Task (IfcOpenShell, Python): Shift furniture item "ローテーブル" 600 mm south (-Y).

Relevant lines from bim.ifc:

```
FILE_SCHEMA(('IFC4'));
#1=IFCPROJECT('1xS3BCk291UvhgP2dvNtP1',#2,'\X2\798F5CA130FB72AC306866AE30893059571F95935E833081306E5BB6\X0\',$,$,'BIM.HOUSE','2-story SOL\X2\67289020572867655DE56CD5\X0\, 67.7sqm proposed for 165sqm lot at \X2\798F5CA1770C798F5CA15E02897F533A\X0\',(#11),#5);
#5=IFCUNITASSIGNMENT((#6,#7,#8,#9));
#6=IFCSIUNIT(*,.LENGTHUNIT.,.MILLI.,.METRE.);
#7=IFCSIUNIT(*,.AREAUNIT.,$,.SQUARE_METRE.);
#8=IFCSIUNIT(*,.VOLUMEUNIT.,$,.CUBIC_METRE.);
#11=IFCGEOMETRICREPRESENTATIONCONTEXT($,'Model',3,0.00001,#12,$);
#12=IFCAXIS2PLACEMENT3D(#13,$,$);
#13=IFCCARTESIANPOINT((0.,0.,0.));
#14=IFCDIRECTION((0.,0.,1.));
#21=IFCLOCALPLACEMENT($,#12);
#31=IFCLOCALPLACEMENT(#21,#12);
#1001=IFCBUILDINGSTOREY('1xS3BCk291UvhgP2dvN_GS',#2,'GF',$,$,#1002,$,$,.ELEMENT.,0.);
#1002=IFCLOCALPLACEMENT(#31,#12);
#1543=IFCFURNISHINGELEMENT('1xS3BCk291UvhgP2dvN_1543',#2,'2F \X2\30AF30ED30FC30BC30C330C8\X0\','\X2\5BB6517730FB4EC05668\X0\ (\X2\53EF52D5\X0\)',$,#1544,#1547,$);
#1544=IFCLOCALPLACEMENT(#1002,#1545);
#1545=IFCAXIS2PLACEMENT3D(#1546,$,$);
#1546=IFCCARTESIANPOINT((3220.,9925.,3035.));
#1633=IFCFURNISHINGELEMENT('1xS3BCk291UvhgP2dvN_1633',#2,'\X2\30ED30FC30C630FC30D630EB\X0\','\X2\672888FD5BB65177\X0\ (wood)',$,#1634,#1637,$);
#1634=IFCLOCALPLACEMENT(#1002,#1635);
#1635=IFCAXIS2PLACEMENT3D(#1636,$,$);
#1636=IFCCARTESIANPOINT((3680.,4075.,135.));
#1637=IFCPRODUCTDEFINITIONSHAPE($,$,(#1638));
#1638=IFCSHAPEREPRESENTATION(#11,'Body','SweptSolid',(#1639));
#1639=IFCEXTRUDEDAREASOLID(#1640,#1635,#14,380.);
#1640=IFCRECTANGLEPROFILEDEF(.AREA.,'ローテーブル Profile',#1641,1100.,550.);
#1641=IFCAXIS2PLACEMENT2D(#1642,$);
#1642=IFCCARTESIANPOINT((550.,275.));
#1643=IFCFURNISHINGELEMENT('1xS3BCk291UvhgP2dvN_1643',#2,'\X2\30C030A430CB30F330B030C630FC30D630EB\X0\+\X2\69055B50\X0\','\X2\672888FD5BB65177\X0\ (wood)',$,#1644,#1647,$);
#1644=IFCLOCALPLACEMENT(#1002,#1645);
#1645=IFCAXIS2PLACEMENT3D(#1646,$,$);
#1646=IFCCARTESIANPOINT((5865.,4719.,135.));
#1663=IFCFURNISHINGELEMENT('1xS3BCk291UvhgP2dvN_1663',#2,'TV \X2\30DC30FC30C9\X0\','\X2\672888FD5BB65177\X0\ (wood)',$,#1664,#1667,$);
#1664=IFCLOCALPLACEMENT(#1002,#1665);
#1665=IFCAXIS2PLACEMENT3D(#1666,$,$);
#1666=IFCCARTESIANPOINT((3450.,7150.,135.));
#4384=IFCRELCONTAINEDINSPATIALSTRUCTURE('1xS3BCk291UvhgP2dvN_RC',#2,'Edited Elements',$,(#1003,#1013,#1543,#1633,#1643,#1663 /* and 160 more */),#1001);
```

```python
import ifcopenshell
import ifcopenshell.api.geometry
import ifcopenshell.util.placement

model = ifcopenshell.open("bim.ifc")

item = model.by_guid("1xS3BCk291UvhgP2dvN_1633")
matrix = ifcopenshell.util.placement.get_local_placement(item.ObjectPlacement)
matrix[1, 3] -= 600.0
ifcopenshell.api.geometry.edit_object_placement(model, product=item, matrix=matrix, is_si=False)

print(ifcopenshell.util.placement.get_local_placement(item.ObjectPlacement).round(3) + 0.0)

model.write("bim_updated.ifc")
```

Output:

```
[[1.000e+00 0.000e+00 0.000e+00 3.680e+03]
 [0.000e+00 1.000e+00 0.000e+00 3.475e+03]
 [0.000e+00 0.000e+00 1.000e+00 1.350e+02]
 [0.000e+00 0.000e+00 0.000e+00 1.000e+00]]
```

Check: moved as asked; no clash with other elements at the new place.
